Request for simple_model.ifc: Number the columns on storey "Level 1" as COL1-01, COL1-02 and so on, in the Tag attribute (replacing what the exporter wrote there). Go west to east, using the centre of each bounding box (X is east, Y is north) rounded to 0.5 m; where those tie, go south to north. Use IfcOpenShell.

First a look at what the model holds.

```python
import ifcopenshell
import ifcopenshell.util.element
import ifcopenshell.util.placement

model = ifcopenshell.open("simple_model.ifc")
print(model.schema)
storey = next(s for s in model.by_type("IfcBuildingStorey") if s.Name == "Level 1")
columns = [e for e in ifcopenshell.util.element.get_decomposition(storey) if e.is_a("IfcColumn")]
for e in sorted(columns, key=lambda e: e.id()):
    origin = ifcopenshell.util.placement.get_local_placement(e.ObjectPlacement)[:3, 3]
    print(e.id(), e.Tag, e.Name, origin.round(2) + 0.0, sep=" | ")
```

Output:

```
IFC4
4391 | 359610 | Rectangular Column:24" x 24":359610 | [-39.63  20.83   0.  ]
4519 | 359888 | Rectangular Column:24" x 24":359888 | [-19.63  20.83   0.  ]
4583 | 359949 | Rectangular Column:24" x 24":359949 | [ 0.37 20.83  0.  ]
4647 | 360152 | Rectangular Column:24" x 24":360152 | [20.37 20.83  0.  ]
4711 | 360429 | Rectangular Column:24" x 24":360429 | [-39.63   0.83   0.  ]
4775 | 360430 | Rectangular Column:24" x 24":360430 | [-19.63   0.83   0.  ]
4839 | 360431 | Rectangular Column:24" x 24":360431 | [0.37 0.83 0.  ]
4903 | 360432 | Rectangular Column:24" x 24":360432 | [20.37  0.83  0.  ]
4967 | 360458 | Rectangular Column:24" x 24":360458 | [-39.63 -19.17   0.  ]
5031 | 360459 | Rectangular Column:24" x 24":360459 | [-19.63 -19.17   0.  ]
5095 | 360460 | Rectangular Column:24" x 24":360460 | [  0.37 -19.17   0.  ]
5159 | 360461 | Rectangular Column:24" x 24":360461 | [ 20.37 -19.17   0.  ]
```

```python
import ifcopenshell
import ifcopenshell.geom
import ifcopenshell.util.element
import ifcopenshell.util.shape

model = ifcopenshell.open("simple_model.ifc")
settings = ifcopenshell.geom.settings()
settings.set("use-world-coords", True)


def centre(element):
    shape = ifcopenshell.geom.create_shape(settings, element)
    return ifcopenshell.util.shape.get_bbox_centroid(shape.geometry)


storey = next(s for s in model.by_type("IfcBuildingStorey") if s.Name == "Level 1")
columns = [e for e in ifcopenshell.util.element.get_decomposition(storey) if e.is_a("IfcColumn")]

# Insertion points can sit at a corner or the storey origin, so sort by the geometry (in metres).
centres = {e: centre(e) for e in columns}
columns.sort(key=lambda e: (round(centres[e][0] / 0.5), centres[e][1]))

for i, e in enumerate(columns, start=1):
    number = f"COL1-{i:02d}"
    e.Tag = number
    print(e.id(), number)

model.write("simple_model_v2.ifc")
```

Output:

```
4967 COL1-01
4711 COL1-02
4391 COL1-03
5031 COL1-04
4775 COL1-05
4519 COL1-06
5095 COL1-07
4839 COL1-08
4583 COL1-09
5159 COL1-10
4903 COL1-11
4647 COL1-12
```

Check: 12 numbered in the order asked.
